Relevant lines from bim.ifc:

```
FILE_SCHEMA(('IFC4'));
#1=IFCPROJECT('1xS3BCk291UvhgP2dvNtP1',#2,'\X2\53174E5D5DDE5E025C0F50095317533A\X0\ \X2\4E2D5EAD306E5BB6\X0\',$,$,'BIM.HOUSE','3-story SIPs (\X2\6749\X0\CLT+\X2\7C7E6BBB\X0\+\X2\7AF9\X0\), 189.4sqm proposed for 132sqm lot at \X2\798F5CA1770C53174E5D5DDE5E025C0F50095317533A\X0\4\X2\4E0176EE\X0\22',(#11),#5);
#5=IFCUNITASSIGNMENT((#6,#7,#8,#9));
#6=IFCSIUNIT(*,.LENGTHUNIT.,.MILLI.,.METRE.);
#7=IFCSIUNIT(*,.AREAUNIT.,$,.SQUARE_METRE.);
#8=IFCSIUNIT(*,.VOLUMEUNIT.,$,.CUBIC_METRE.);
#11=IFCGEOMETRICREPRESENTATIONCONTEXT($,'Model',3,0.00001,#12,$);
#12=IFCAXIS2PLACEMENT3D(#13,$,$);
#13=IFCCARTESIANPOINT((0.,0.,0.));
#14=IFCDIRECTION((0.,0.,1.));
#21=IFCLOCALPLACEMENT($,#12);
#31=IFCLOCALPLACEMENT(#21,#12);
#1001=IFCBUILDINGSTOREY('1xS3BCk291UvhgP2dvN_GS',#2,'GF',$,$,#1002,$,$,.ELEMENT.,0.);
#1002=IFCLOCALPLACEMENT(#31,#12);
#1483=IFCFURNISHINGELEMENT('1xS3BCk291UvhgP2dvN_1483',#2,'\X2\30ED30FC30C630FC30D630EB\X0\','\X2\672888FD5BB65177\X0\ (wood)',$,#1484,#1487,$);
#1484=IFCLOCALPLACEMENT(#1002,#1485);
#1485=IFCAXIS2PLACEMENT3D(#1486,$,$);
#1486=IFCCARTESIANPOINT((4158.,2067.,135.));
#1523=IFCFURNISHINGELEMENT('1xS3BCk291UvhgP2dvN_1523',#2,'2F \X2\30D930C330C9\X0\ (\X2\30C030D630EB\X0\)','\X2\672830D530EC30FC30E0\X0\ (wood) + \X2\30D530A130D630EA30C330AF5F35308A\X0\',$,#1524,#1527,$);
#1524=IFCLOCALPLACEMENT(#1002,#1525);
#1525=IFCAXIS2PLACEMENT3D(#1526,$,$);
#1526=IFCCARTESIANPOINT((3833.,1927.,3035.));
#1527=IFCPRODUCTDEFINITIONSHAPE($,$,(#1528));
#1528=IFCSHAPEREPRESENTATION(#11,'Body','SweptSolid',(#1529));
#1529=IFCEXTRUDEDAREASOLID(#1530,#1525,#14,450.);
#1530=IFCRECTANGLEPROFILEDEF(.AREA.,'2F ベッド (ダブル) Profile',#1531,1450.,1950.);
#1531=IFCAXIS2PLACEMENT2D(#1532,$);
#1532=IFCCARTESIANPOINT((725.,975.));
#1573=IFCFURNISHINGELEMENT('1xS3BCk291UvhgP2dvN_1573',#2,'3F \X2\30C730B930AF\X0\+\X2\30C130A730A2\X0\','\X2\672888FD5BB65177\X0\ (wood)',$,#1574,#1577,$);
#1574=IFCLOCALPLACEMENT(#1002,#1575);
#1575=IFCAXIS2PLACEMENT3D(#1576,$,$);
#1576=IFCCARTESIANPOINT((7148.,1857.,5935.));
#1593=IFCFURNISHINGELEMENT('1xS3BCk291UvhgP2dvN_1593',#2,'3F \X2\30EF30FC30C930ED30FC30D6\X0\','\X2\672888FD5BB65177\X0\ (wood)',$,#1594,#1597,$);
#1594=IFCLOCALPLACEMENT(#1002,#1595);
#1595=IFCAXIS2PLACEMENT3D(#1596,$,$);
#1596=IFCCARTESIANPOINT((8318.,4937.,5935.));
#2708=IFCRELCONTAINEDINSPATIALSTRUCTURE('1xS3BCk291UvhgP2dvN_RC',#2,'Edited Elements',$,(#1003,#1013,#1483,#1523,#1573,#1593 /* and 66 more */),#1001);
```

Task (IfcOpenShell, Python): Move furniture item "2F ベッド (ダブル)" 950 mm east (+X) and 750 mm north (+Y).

```python
import ifcopenshell
import ifcopenshell.api.geometry
import ifcopenshell.util.placement
import ifcopenshell.util.unit

model = ifcopenshell.open("bim.ifc")
unit_scale = ifcopenshell.util.unit.calculate_unit_scale(model)

item = model.by_guid("1xS3BCk291UvhgP2dvN_1523")
matrix = ifcopenshell.util.placement.get_local_placement(item.ObjectPlacement)
matrix[0, 3] += 0.95 / unit_scale
matrix[1, 3] += 0.75 / unit_scale
ifcopenshell.api.geometry.edit_object_placement(model, product=item, matrix=matrix, is_si=False)

print(ifcopenshell.util.placement.get_local_placement(item.ObjectPlacement).round(3) + 0.0)

model.write("bim_rev.ifc")
```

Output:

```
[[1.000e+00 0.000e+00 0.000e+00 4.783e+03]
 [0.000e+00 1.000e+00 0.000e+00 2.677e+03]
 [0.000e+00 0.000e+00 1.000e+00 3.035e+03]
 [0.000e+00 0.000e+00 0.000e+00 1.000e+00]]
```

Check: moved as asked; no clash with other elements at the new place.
